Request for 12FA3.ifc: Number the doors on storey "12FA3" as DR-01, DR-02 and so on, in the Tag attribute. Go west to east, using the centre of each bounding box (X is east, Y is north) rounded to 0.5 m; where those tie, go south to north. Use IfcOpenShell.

First a look at what the model holds.

```python
import ifcopenshell
import ifcopenshell.util.element
import ifcopenshell.util.placement

model = ifcopenshell.open("12FA3.ifc")
print(model.schema)
storey = next(s for s in model.by_type("IfcBuildingStorey") if s.Name == "12FA3")
doors = [e for e in ifcopenshell.util.element.get_decomposition(storey) if e.is_a("IfcDoor")]
for e in sorted(doors, key=lambda e: e.id()):
    origin = ifcopenshell.util.placement.get_local_placement(e.ObjectPlacement)[:3, 3]
    print(e.id(), e.Tag, e.Name, origin.round(2) + 0.0, sep=" | ")
```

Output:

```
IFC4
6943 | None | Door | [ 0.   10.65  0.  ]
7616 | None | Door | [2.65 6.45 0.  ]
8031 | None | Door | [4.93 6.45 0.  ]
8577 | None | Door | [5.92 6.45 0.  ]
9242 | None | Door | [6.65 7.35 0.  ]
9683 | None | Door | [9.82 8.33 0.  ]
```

```python
import ifcopenshell
import ifcopenshell.geom
import ifcopenshell.util.element
import ifcopenshell.util.shape

model = ifcopenshell.open("12FA3.ifc")
settings = ifcopenshell.geom.settings()
settings.set("use-world-coords", True)


def centre(element):
    shape = ifcopenshell.geom.create_shape(settings, element)
    return ifcopenshell.util.shape.get_bbox_centroid(shape.geometry)


storey = next(s for s in model.by_type("IfcBuildingStorey") if s.Name == "12FA3")
doors = [e for e in ifcopenshell.util.element.get_decomposition(storey) if e.is_a("IfcDoor")]

# Insertion points can sit at a corner or the storey origin, so sort by the geometry (in metres).
centres = {e: centre(e) for e in doors}
doors.sort(key=lambda e: (round(centres[e][0] / 0.5), centres[e][1]))

for i, e in enumerate(doors, start=1):
    number = f"DR-{i:02d}"
    e.Tag = number
    print(e.id(), number)

model.write("12FA3_edited.ifc")
```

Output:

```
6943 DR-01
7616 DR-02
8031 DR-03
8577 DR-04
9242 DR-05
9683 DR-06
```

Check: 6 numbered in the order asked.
